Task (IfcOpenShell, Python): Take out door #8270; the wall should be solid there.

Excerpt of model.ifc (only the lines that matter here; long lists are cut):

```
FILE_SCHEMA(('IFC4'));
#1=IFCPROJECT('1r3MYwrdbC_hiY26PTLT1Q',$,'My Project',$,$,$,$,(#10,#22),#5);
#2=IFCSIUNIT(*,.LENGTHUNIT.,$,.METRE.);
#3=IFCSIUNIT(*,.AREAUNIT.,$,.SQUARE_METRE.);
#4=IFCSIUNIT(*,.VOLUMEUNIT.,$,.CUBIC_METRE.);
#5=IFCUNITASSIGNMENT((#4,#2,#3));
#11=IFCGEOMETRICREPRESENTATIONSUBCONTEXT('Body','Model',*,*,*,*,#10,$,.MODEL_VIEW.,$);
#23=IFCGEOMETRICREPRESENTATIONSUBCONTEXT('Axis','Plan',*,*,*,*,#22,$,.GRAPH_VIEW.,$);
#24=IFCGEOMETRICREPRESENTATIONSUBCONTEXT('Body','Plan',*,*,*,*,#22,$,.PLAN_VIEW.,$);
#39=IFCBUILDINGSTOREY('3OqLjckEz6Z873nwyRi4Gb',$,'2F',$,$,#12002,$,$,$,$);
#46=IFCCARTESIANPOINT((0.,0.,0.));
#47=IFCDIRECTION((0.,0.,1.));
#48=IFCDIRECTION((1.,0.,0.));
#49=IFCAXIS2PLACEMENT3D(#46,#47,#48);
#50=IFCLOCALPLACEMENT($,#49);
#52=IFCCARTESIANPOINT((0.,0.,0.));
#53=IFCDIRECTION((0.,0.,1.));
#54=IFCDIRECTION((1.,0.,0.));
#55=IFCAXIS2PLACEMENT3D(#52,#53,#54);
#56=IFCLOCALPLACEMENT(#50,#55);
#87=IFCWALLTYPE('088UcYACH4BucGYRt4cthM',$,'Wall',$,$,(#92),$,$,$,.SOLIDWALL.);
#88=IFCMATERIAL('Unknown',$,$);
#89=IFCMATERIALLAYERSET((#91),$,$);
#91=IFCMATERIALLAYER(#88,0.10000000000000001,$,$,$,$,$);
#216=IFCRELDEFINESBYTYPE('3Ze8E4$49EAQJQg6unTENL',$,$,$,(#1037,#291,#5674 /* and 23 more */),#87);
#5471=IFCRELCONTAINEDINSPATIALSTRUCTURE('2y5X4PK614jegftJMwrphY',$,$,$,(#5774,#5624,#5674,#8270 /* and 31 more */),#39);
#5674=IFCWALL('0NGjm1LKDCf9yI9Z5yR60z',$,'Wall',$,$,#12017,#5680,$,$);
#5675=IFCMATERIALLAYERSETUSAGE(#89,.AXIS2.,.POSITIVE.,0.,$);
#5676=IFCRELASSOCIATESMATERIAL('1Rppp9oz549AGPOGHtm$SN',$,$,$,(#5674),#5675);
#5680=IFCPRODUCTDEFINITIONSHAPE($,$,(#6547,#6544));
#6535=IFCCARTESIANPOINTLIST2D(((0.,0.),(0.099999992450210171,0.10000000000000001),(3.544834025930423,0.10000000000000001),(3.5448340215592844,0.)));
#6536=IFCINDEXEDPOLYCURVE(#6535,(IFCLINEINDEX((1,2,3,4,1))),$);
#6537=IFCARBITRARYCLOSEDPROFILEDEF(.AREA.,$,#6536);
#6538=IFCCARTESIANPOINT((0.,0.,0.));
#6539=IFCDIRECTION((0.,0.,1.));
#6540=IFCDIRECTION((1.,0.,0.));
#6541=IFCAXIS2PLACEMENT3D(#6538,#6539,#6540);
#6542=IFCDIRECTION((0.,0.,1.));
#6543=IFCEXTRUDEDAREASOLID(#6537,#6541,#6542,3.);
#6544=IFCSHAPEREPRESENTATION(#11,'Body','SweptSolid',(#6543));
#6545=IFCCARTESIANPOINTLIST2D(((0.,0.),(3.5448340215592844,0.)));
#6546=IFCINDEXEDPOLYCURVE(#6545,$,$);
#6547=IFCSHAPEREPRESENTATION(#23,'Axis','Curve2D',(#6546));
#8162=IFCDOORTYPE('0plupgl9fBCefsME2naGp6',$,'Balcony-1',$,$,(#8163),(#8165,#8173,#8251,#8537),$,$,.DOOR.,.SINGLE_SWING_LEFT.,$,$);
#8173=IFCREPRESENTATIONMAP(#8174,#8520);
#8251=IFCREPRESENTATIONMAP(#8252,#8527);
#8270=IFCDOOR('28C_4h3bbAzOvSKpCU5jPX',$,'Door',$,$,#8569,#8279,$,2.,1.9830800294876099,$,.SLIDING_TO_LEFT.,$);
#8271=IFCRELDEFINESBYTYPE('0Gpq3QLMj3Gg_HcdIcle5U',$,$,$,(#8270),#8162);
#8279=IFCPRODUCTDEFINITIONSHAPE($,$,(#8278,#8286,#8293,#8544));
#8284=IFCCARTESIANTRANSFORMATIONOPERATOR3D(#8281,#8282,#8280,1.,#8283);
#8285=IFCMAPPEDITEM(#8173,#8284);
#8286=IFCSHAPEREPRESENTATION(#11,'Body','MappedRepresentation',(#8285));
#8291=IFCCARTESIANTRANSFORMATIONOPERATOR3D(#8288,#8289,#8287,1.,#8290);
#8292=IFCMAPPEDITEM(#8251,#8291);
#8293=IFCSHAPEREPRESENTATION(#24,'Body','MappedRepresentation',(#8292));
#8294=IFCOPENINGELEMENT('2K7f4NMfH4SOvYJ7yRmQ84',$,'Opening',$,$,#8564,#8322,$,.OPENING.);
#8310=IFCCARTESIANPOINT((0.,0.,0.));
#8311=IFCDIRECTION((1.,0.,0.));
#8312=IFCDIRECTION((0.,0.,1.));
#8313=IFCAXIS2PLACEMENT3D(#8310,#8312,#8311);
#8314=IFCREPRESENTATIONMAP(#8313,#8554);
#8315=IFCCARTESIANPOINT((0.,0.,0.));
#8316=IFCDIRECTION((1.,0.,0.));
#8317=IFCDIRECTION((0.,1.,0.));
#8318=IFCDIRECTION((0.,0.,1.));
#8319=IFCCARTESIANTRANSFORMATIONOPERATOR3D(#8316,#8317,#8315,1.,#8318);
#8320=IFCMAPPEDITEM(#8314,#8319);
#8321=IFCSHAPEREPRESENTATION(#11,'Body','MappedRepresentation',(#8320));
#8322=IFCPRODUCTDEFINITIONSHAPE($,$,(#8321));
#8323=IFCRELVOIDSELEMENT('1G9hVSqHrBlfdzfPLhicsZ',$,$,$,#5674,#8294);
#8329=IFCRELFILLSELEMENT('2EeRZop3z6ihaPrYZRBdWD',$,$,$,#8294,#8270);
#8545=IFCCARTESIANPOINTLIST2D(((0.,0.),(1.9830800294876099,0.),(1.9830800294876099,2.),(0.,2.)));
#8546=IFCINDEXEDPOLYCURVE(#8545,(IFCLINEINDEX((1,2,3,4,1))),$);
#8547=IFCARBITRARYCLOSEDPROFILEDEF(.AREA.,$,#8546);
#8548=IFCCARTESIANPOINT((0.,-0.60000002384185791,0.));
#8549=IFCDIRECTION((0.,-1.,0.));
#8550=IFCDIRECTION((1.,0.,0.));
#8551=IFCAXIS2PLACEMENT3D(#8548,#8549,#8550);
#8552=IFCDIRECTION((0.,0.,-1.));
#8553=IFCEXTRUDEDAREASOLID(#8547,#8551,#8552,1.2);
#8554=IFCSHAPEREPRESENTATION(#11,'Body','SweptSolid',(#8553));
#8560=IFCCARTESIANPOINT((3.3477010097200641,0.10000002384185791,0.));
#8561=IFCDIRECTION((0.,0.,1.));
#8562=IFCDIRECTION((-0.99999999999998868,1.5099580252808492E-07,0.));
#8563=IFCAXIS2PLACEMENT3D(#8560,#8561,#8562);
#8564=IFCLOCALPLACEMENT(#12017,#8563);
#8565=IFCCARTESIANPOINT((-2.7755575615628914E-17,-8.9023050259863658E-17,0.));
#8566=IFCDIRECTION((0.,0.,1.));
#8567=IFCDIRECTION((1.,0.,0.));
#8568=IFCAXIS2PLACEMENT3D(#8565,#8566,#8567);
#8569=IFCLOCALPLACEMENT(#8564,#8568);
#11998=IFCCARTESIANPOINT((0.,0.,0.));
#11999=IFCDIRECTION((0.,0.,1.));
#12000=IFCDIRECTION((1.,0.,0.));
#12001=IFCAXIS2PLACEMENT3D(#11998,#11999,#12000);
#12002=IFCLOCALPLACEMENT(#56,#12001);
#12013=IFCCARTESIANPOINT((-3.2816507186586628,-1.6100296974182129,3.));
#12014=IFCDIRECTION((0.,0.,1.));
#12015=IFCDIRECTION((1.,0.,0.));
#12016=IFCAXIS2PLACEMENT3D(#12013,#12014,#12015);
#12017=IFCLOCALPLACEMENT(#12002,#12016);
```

```python
import ifcopenshell
import ifcopenshell.api.feature
import ifcopenshell.api.root
import ifcopenshell.geom
import ifcopenshell.util.shape

model = ifcopenshell.open("model.ifc")
settings = ifcopenshell.geom.settings()


def volume(element):
    """Net volume in cubic metres, openings subtracted."""
    shape = ifcopenshell.geom.create_shape(settings, element)
    return ifcopenshell.util.shape.get_volume(shape.geometry)


door = model.by_id(8270)
opening = door.FillsVoids[0].RelatingOpeningElement
wall = opening.VoidsElements[0].RelatingBuildingElement
before = volume(wall)

ifcopenshell.api.root.remove_product(model, product=door)
ifcopenshell.api.feature.remove_feature(model, feature=opening)

after = volume(wall)

print(f"wall volume {before:.3f} -> {after:.3f} m3")

model.write("model_v2.ifc")
```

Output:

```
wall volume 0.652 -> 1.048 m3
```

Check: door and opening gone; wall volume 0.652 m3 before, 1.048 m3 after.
